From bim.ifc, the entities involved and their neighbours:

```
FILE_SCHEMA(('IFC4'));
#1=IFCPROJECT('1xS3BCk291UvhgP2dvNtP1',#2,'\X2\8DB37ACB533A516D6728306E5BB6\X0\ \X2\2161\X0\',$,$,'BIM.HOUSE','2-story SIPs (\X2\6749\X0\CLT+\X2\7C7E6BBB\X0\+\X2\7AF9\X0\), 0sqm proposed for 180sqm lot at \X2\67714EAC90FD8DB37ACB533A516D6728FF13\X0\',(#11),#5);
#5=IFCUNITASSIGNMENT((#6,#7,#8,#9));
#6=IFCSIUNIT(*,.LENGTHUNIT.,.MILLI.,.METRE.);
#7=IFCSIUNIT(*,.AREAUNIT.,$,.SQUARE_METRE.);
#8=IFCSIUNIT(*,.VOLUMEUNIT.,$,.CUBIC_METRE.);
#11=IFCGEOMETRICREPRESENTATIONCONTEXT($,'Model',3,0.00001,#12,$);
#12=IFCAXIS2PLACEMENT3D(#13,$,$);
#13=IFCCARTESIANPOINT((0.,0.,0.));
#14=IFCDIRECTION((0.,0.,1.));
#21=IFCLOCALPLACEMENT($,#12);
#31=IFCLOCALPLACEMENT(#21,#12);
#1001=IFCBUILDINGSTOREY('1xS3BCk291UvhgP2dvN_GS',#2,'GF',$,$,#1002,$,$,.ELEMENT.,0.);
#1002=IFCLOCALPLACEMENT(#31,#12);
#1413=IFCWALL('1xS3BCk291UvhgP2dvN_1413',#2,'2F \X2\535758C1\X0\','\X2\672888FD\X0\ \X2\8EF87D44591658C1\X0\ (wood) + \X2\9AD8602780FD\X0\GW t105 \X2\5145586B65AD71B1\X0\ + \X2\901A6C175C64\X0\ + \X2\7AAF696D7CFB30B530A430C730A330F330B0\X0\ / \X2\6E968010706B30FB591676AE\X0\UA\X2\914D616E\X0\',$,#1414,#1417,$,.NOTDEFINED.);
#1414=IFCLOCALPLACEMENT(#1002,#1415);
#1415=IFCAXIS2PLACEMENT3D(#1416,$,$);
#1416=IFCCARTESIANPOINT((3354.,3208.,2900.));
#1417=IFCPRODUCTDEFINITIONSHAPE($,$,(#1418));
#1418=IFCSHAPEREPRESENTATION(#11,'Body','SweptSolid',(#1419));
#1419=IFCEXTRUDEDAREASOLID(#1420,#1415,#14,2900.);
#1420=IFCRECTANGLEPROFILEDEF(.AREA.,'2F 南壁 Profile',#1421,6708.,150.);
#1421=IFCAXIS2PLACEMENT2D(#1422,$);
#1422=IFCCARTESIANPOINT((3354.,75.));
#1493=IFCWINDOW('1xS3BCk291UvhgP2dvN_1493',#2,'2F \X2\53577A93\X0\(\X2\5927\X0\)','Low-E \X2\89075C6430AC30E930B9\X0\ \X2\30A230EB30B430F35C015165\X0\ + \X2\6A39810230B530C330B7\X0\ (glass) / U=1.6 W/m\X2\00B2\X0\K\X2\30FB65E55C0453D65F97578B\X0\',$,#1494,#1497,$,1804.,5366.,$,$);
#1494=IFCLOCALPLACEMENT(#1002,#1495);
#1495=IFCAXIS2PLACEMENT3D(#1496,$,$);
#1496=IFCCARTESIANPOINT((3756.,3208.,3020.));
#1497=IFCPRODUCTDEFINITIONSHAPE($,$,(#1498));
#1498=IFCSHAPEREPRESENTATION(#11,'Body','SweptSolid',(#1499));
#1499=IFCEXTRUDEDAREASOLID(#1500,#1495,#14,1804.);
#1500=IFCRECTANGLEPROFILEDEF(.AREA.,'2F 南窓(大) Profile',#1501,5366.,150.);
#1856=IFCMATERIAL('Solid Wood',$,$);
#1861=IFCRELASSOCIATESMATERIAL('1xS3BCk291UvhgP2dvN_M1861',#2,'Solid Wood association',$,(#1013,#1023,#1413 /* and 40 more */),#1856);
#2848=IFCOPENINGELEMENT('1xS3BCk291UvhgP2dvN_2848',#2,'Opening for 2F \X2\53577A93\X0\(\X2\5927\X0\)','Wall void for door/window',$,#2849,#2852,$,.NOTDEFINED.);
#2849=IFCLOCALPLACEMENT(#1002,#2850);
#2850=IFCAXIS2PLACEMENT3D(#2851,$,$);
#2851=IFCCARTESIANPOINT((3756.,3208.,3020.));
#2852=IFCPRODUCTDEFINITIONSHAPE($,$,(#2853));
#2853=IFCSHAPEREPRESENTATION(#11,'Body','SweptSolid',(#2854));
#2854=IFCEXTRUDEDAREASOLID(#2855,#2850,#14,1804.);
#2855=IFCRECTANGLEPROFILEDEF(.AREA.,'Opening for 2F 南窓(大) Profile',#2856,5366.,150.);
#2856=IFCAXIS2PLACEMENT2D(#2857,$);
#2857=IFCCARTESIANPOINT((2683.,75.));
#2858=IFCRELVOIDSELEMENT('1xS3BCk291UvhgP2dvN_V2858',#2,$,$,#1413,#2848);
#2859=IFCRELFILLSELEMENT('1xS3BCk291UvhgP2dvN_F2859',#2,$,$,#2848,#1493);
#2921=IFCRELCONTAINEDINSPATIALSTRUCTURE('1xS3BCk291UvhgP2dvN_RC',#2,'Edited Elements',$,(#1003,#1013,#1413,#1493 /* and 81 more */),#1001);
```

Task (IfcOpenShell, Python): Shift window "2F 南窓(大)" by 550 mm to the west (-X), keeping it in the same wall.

```python
import ifcopenshell
import ifcopenshell.api.geometry
import ifcopenshell.util.placement
import ifcopenshell.util.unit

model = ifcopenshell.open("bim.ifc")
unit_scale = ifcopenshell.util.unit.calculate_unit_scale(model)

window = model.by_id(1493)
opening = window.FillsVoids[0].RelatingOpeningElement
wall = opening.VoidsElements[0].RelatingBuildingElement

wall_matrix = ifcopenshell.util.placement.get_local_placement(wall.ObjectPlacement)
shift = wall_matrix[:3, 0] * -0.55 / unit_scale
before = ifcopenshell.util.placement.get_local_placement(window.ObjectPlacement)[:3, 3].copy()

# The window is not placed relative to its opening, so move both.
for product in (opening, window):
    matrix = ifcopenshell.util.placement.get_local_placement(product.ObjectPlacement)
    matrix[:3, 3] += shift
    ifcopenshell.api.geometry.edit_object_placement(model, product=product, matrix=matrix, is_si=False)

after = ifcopenshell.util.placement.get_local_placement(window.ObjectPlacement)[:3, 3]
print("window moved by", (after - before).round(3) + 0.0)

model.write("bim_updated.ifc")
```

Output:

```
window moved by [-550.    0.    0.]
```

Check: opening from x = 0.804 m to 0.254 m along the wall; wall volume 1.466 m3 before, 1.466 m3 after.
